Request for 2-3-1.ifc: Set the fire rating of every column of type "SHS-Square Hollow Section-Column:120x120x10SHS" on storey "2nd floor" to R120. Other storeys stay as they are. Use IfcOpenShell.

First a look at what the model holds.

```python
import ifcopenshell
import ifcopenshell.util.element

model = ifcopenshell.open("2-3-1.ifc")
print(model.schema)
storey = next(s for s in model.by_type("IfcBuildingStorey") if s.Name == "2nd floor")
columns = [e for e in ifcopenshell.util.element.get_decomposition(storey) if e.is_a("IfcColumn")]
seen = {}
for e in columns:
    element_type = ifcopenshell.util.element.get_type(e)
    key = (element_type.Name if element_type != e and element_type else None, ifcopenshell.util.element.get_pset(e, "Pset_ColumnCommon", "FireRating"))
    seen[key] = seen.get(key, 0) + 1
for (name, value), count in sorted(seen.items(), key=str):
    print(count, "x", name, "|", value)
```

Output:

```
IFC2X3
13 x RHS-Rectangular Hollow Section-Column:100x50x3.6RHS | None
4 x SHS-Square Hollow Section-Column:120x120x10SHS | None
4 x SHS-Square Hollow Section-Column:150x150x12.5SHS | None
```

```python
import ifcopenshell
import ifcopenshell.api.pset
import ifcopenshell.util.element

model = ifcopenshell.open("2-3-1.ifc")

storey = next(s for s in model.by_type("IfcBuildingStorey") if s.Name == "2nd floor")
columns = [e for e in ifcopenshell.util.element.get_decomposition(storey) if e.is_a("IfcColumn")]

count = 0
for e in columns:
    element_type = ifcopenshell.util.element.get_type(e)
    if element_type in (None, e) or element_type.Name != "SHS-Square Hollow Section-Column:120x120x10SHS":
        continue
    # add_pset returns the element's existing set when there is one.
    pset = ifcopenshell.api.pset.add_pset(model, product=e, name="Pset_ColumnCommon")
    ifcopenshell.api.pset.edit_pset(model, pset=pset, properties={"FireRating": "R120"})
    count += 1

print(count, "columns updated")

model.write("2-3-1_rev.ifc")
```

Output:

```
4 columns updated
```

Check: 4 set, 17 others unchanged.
